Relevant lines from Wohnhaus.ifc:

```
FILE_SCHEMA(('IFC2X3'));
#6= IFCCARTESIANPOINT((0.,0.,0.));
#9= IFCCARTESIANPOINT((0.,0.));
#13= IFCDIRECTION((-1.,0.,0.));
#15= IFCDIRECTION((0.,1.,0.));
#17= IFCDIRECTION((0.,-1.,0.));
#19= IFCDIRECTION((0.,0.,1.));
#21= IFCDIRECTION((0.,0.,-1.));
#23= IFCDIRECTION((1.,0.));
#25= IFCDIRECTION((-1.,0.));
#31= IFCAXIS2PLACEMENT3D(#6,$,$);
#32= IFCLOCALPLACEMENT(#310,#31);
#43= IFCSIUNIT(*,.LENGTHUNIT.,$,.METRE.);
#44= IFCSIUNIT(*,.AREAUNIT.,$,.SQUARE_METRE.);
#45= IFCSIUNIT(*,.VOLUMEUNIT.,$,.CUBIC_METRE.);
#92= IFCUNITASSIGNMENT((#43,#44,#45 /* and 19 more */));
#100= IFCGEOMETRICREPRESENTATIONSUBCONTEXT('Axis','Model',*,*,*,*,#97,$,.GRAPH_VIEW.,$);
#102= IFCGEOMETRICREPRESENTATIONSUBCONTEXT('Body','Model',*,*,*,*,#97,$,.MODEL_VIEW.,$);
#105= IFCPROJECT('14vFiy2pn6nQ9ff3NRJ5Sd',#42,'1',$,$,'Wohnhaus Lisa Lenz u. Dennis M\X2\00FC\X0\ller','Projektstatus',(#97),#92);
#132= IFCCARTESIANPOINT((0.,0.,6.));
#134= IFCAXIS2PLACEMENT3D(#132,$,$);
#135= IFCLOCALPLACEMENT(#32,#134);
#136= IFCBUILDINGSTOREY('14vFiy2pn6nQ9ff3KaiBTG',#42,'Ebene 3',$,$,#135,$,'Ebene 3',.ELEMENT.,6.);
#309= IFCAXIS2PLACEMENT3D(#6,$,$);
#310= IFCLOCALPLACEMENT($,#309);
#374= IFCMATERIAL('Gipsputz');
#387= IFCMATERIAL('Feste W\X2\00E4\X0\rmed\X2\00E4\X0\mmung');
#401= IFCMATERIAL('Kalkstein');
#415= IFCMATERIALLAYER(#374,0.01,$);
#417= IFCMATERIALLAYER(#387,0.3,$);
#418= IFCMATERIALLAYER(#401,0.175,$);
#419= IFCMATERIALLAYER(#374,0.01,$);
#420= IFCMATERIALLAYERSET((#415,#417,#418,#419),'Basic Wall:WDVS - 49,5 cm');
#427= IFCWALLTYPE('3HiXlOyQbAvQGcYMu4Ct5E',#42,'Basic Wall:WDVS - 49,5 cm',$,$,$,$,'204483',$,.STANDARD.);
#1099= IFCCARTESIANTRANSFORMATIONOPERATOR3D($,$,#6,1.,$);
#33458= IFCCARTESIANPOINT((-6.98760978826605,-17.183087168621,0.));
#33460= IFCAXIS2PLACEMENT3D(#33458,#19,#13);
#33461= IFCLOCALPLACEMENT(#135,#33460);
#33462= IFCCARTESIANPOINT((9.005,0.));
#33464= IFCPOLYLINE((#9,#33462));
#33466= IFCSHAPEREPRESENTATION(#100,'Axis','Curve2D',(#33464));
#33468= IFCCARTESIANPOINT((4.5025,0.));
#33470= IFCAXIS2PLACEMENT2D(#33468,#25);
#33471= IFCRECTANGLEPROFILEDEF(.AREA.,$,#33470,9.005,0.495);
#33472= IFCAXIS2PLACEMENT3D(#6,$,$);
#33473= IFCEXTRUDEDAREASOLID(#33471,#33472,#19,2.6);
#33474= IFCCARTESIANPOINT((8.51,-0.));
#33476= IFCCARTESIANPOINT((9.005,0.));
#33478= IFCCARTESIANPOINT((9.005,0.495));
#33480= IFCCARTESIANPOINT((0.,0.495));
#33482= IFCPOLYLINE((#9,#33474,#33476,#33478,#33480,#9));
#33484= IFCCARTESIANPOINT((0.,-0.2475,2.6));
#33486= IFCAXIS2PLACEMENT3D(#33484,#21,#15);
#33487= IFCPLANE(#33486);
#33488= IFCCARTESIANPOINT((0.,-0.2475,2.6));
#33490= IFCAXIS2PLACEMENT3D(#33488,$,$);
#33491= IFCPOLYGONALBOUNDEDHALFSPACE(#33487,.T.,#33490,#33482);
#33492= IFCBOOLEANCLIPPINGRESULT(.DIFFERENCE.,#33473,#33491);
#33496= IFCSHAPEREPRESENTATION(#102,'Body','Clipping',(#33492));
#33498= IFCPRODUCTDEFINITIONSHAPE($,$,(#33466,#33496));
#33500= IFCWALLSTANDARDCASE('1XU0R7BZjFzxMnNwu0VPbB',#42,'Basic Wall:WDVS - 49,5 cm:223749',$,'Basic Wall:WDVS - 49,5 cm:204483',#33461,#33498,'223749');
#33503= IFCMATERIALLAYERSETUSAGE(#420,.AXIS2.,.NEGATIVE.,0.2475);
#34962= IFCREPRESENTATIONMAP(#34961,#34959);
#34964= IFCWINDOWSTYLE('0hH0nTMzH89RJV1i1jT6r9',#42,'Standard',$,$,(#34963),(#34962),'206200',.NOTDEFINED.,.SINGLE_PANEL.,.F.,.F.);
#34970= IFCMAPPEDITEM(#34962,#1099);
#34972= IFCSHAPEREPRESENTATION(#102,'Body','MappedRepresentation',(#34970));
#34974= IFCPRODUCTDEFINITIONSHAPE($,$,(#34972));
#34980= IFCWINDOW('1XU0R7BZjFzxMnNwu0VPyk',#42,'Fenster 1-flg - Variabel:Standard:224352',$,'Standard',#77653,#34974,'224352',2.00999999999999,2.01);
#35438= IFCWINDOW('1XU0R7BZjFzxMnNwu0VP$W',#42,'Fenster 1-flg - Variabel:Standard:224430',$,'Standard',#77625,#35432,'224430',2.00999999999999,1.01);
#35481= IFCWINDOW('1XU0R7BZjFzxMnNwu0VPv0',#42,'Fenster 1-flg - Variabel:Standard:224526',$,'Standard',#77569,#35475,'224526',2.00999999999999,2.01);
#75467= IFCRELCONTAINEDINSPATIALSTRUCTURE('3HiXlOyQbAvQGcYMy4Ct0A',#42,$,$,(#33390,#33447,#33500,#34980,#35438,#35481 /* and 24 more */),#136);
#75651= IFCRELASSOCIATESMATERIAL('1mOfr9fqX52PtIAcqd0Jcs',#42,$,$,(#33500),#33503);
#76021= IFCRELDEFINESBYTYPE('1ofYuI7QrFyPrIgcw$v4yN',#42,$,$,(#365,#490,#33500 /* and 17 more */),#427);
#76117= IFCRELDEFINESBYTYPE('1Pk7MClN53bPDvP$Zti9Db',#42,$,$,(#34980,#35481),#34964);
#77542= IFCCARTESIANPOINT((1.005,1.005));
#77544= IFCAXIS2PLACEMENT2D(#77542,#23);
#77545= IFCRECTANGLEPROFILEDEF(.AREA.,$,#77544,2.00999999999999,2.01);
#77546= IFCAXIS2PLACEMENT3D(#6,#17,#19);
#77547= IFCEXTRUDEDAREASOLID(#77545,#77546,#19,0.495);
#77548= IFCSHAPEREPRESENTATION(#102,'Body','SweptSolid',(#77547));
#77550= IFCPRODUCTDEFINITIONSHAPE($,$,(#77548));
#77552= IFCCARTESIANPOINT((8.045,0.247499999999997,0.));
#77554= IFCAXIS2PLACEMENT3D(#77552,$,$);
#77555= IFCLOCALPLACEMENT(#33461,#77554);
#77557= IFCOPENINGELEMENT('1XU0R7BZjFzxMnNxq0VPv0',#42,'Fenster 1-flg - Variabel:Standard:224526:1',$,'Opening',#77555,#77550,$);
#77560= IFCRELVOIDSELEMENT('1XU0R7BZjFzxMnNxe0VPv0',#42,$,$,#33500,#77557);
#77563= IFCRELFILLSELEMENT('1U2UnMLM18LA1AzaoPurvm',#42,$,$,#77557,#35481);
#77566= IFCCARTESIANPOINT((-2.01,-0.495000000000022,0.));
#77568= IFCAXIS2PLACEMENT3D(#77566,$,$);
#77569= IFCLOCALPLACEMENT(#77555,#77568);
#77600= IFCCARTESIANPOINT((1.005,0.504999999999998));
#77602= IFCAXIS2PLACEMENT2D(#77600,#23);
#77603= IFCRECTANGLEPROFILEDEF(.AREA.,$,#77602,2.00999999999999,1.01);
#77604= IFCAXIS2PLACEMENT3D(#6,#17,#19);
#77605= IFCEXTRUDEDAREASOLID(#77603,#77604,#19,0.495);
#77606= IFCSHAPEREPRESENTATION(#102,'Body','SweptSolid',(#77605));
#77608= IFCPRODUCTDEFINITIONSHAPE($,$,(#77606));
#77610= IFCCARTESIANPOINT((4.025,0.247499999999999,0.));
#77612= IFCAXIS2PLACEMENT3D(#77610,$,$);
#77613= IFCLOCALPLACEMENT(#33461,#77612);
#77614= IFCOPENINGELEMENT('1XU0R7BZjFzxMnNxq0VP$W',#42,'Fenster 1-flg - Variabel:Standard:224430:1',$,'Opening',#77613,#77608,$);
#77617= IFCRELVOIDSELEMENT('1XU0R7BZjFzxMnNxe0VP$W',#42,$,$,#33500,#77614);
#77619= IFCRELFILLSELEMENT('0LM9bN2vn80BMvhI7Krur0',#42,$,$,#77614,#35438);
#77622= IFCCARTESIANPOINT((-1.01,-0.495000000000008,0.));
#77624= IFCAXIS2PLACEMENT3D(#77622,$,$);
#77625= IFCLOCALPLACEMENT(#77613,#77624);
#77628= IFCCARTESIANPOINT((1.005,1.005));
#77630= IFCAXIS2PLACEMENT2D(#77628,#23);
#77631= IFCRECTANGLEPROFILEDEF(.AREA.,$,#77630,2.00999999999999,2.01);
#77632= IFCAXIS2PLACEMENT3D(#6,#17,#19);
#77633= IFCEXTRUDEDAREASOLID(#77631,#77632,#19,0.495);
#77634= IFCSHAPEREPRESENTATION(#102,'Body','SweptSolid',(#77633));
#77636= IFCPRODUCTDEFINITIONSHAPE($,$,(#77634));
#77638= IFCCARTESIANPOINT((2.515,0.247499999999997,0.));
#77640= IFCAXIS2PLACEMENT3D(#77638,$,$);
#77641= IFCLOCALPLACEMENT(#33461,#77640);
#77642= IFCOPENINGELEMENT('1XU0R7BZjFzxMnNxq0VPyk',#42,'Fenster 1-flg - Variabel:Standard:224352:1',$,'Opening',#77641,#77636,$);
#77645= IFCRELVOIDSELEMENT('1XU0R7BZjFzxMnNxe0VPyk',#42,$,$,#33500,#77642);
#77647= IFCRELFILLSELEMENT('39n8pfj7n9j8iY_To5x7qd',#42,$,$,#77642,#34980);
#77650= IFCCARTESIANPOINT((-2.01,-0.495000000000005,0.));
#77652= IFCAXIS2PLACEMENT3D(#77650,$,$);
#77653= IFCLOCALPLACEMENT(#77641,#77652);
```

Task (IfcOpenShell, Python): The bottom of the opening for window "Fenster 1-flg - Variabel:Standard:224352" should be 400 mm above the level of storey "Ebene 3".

```python
import numpy as np
import ifcopenshell
import ifcopenshell.api.geometry
import ifcopenshell.geom
import ifcopenshell.util.element
import ifcopenshell.util.placement
import ifcopenshell.util.shape
import ifcopenshell.util.unit

model = ifcopenshell.open("Wohnhaus.ifc")
unit_scale = ifcopenshell.util.unit.calculate_unit_scale(model)

window = model.by_id(34980)
opening = window.FillsVoids[0].RelatingOpeningElement
storey = ifcopenshell.util.element.get_container(window, ifc_class="IfcBuildingStorey")
level = ifcopenshell.util.placement.get_local_placement(storey.ObjectPlacement)[2, 3]

# The opening's origin need not be at the sill, so measure its lowest point.
shape = ifcopenshell.geom.create_shape(ifcopenshell.geom.settings(), opening)
bottom = ifcopenshell.util.shape.get_shape_bottom_elevation(shape, shape.geometry) / unit_scale
dz = level + 0.4 - bottom

shift = np.array([0.0, 0.0, dz])
# The window is placed relative to its opening, so it follows when the opening moves.
matrix = ifcopenshell.util.placement.get_local_placement(opening.ObjectPlacement)
matrix[:3, 3] += shift
ifcopenshell.api.geometry.edit_object_placement(
    model, product=opening, matrix=matrix, is_si=False, should_transform_children=True
)

print(f"moved by {dz * unit_scale:+.3f} m")

model.write("Wohnhaus-out.ifc")
```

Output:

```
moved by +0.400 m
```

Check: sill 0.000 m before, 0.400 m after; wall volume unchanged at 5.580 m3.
